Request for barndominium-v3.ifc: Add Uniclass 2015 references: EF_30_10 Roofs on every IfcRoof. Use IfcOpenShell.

First a look at what the model holds.

```python
import ifcopenshell

model = ifcopenshell.open("barndominium-v3.ifc")
print(model.schema)
print("classifications:", [c.Name for c in model.by_type("IfcClassification")])
for ifc_class in ("IfcDoor", "IfcRoof", "IfcStair", "IfcWall", "IfcWindow"):
    print(ifc_class, len(model.by_type(ifc_class)))
```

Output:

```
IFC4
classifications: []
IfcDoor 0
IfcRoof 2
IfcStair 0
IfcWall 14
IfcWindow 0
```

```python
import ifcopenshell
import ifcopenshell.api.classification

model = ifcopenshell.open("barndominium-v3.ifc")

system = ifcopenshell.api.classification.add_classification(model, classification="Uniclass 2015")

codes = {
    "IfcRoof": ("EF_30_10", "Roofs"),
}
for ifc_class, (code, name) in codes.items():
    products = model.by_type(ifc_class)
    ifcopenshell.api.classification.add_reference(
        model, products=products, classification=system, identification=code, name=name
    )
    print(code, len(products))

model.write("barndominium-v3-out.ifc")
```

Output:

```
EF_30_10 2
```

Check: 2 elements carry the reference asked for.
